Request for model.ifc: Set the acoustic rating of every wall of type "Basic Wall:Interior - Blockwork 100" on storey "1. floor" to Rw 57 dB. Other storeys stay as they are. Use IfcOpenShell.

First a look at what the model holds.

```python
import ifcopenshell
import ifcopenshell.util.element

model = ifcopenshell.open("model.ifc")
print(model.schema)
storey = next(s for s in model.by_type("IfcBuildingStorey") if s.Name == "1. floor")
walls = [e for e in ifcopenshell.util.element.get_decomposition(storey) if e.is_a("IfcWall")]
seen = {}
for e in walls:
    element_type = ifcopenshell.util.element.get_type(e)
    key = (element_type.Name if element_type != e and element_type else None, ifcopenshell.util.element.get_pset(e, "Pset_WallCommon", "AcousticRating"))
    seen[key] = seen.get(key, 0) + 1
for (name, value), count in sorted(seen.items(), key=str):
    print(count, "x", name, "|", value)
```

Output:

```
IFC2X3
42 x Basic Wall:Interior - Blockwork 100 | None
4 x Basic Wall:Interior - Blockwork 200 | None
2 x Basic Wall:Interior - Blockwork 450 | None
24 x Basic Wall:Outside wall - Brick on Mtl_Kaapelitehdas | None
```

```python
import ifcopenshell
import ifcopenshell.api.pset
import ifcopenshell.util.element

model = ifcopenshell.open("model.ifc")

storey = next(s for s in model.by_type("IfcBuildingStorey") if s.Name == "1. floor")
walls = [e for e in ifcopenshell.util.element.get_decomposition(storey) if e.is_a("IfcWall")]

count = 0
for e in walls:
    element_type = ifcopenshell.util.element.get_type(e)
    if element_type in (None, e) or element_type.Name != "Basic Wall:Interior - Blockwork 100":
        continue
    # add_pset returns the element's existing set when there is one.
    pset = ifcopenshell.api.pset.add_pset(model, product=e, name="Pset_WallCommon")
    ifcopenshell.api.pset.edit_pset(model, pset=pset, properties={"AcousticRating": "Rw 57 dB"})
    count += 1

print(count, "walls updated")

model.write("model_edited.ifc")
```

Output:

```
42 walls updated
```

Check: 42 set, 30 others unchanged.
